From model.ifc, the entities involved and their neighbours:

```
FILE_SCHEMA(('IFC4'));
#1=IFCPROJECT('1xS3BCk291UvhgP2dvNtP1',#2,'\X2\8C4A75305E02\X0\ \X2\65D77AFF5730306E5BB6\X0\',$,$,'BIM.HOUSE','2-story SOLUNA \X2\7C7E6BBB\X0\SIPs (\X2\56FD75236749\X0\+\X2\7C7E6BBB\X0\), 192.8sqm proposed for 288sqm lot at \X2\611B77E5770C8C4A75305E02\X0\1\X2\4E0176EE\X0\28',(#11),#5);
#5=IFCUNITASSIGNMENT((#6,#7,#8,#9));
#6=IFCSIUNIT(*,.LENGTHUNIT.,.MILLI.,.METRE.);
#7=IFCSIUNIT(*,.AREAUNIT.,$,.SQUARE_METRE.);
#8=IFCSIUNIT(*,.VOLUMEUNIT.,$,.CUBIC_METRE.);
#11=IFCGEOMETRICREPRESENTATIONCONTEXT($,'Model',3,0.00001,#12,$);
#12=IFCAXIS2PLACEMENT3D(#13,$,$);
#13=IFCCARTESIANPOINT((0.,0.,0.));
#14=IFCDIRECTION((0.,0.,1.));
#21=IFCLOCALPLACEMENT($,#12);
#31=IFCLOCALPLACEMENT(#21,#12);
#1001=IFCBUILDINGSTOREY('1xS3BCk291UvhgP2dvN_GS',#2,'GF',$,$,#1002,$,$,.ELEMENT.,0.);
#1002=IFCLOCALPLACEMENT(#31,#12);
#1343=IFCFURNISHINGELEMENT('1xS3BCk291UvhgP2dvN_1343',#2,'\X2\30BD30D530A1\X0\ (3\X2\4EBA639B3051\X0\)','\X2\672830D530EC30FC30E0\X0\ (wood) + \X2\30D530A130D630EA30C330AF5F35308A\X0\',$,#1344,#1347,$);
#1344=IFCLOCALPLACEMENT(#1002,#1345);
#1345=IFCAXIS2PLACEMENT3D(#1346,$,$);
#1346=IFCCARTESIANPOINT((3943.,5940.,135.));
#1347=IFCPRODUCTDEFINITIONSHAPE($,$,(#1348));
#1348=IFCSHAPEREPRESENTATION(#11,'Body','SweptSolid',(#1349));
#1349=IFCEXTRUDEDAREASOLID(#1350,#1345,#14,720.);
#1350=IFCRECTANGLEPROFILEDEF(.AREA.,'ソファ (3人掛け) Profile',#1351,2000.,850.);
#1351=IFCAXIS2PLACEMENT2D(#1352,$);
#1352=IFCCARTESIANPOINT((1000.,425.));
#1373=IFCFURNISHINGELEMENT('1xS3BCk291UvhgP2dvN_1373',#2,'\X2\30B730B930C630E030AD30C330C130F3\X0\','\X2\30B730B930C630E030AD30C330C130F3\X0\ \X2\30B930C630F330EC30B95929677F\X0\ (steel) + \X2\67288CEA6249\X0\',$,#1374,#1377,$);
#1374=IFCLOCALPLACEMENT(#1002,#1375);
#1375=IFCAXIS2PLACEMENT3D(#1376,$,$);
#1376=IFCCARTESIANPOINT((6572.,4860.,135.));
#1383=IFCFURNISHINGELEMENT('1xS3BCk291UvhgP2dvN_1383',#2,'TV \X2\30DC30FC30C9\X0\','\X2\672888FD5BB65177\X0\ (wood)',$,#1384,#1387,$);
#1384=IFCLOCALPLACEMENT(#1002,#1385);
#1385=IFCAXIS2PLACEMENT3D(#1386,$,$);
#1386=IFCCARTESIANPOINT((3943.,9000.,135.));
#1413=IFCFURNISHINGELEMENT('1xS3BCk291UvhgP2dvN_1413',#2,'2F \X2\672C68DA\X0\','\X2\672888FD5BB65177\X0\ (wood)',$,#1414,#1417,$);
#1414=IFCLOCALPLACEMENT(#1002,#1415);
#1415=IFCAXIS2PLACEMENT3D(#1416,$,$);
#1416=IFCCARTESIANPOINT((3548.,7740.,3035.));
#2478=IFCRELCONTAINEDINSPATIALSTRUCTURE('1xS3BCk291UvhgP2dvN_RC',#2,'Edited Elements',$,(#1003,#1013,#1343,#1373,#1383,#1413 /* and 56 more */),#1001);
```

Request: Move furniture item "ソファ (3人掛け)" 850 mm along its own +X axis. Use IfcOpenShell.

```python
import ifcopenshell
import ifcopenshell.api.geometry
import ifcopenshell.util.placement
import ifcopenshell.util.unit

model = ifcopenshell.open("model.ifc")
unit_scale = ifcopenshell.util.unit.calculate_unit_scale(model)

item = model.by_guid("1xS3BCk291UvhgP2dvN_1343")
matrix = ifcopenshell.util.placement.get_local_placement(item.ObjectPlacement)
matrix[:3, 3] += matrix[:3, 0] * 0.85 / unit_scale
ifcopenshell.api.geometry.edit_object_placement(model, product=item, matrix=matrix, is_si=False)

print(ifcopenshell.util.placement.get_local_placement(item.ObjectPlacement).round(3) + 0.0)

model.write("model-out.ifc")
```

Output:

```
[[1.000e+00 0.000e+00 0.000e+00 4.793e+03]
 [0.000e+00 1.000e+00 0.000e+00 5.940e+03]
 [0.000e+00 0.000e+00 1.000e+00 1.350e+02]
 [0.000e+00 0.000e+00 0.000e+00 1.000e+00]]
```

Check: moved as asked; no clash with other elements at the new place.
